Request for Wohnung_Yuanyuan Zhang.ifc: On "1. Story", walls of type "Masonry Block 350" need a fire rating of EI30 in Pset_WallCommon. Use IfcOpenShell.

First a look at what the model holds.

```python
import ifcopenshell
import ifcopenshell.util.element

model = ifcopenshell.open("Wohnung_Yuanyuan Zhang.ifc")
print(model.schema)
storey = next(s for s in model.by_type("IfcBuildingStorey") if s.Name == "1. Story")
walls = [e for e in ifcopenshell.util.element.get_decomposition(storey) if e.is_a("IfcWall")]
seen = {}
for e in walls:
    element_type = ifcopenshell.util.element.get_type(e)
    key = (element_type.Name if element_type != e and element_type else None, ifcopenshell.util.element.get_pset(e, "Pset_WallCommon", "FireRating"))
    seen[key] = seen.get(key, 0) + 1
for (name, value), count in sorted(seen.items(), key=str):
    print(count, "x", name, "|", value)
```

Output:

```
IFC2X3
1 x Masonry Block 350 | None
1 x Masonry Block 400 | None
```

```python
import ifcopenshell
import ifcopenshell.api.pset
import ifcopenshell.util.element

model = ifcopenshell.open("Wohnung_Yuanyuan Zhang.ifc")

storey = next(s for s in model.by_type("IfcBuildingStorey") if s.Name == "1. Story")
walls = [e for e in ifcopenshell.util.element.get_decomposition(storey) if e.is_a("IfcWall")]

count = 0
for e in walls:
    element_type = ifcopenshell.util.element.get_type(e)
    if element_type in (None, e) or element_type.Name != "Masonry Block 350":
        continue
    # add_pset returns the element's existing set when there is one.
    pset = ifcopenshell.api.pset.add_pset(model, product=e, name="Pset_WallCommon")
    ifcopenshell.api.pset.edit_pset(model, pset=pset, properties={"FireRating": "EI30"})
    count += 1

print(count, "walls updated")

model.write("Wohnung_Yuanyuan Zhang_edited.ifc")
```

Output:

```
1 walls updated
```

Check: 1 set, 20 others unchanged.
